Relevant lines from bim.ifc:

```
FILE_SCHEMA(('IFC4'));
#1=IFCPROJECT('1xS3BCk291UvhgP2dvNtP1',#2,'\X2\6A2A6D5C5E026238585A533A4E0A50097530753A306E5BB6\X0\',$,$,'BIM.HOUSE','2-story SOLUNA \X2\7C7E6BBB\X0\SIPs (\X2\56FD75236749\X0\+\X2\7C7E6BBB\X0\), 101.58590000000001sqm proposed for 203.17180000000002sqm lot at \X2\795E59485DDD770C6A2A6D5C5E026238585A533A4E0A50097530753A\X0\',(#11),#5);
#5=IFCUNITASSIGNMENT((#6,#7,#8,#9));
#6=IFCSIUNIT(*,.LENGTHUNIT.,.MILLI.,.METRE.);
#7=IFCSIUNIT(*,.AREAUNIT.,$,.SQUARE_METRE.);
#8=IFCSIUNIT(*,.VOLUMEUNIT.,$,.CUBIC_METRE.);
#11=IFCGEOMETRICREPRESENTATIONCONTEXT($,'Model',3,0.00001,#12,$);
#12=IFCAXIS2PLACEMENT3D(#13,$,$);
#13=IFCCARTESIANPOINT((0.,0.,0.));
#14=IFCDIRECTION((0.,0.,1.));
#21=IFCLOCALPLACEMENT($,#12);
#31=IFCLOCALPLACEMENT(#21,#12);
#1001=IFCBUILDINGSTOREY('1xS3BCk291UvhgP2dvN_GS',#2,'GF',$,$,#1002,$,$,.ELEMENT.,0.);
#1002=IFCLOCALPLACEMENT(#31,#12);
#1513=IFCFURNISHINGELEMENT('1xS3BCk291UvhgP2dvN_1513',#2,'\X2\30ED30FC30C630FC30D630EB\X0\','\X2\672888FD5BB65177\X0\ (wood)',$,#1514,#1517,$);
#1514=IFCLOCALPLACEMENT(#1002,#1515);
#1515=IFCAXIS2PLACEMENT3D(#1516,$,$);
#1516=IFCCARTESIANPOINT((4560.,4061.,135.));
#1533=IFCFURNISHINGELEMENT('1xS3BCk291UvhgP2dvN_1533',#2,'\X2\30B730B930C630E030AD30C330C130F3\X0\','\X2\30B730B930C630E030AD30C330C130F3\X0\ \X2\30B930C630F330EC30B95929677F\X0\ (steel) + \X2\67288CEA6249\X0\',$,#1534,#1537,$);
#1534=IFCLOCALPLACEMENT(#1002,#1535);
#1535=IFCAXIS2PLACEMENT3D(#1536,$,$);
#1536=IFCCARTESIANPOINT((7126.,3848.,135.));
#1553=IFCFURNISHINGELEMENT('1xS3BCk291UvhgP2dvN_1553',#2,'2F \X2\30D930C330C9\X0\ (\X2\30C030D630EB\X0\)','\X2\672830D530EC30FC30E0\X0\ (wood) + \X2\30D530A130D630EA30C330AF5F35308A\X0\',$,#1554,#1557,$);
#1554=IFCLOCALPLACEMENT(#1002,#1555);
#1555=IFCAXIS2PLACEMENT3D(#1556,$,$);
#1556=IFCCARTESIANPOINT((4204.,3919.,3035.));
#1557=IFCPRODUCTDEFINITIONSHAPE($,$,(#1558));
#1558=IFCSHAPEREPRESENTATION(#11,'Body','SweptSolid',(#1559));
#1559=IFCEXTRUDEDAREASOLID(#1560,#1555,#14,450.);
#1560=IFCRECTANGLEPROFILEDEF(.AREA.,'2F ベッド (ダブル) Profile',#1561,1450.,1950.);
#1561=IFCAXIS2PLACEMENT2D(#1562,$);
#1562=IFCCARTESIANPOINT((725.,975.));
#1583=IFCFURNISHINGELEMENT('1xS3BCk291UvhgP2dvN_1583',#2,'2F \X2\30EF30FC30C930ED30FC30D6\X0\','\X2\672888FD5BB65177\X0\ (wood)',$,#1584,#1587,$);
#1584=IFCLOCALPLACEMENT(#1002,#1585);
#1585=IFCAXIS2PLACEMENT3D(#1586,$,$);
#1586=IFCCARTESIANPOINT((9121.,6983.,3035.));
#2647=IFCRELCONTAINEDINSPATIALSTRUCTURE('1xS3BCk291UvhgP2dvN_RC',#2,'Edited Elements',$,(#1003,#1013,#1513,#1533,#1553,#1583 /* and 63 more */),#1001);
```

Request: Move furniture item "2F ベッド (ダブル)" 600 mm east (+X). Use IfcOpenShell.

```python
import ifcopenshell
import ifcopenshell.api.geometry
import ifcopenshell.util.placement

model = ifcopenshell.open("bim.ifc")

item = model.by_guid("1xS3BCk291UvhgP2dvN_1553")
matrix = ifcopenshell.util.placement.get_local_placement(item.ObjectPlacement)
matrix[0, 3] += 600.0
ifcopenshell.api.geometry.edit_object_placement(model, product=item, matrix=matrix, is_si=False)

print(ifcopenshell.util.placement.get_local_placement(item.ObjectPlacement).round(3) + 0.0)

model.write("bim_rev.ifc")
```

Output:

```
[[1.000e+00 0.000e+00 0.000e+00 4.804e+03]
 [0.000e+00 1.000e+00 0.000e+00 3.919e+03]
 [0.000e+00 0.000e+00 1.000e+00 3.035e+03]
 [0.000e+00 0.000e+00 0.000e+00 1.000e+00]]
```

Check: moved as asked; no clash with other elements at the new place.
